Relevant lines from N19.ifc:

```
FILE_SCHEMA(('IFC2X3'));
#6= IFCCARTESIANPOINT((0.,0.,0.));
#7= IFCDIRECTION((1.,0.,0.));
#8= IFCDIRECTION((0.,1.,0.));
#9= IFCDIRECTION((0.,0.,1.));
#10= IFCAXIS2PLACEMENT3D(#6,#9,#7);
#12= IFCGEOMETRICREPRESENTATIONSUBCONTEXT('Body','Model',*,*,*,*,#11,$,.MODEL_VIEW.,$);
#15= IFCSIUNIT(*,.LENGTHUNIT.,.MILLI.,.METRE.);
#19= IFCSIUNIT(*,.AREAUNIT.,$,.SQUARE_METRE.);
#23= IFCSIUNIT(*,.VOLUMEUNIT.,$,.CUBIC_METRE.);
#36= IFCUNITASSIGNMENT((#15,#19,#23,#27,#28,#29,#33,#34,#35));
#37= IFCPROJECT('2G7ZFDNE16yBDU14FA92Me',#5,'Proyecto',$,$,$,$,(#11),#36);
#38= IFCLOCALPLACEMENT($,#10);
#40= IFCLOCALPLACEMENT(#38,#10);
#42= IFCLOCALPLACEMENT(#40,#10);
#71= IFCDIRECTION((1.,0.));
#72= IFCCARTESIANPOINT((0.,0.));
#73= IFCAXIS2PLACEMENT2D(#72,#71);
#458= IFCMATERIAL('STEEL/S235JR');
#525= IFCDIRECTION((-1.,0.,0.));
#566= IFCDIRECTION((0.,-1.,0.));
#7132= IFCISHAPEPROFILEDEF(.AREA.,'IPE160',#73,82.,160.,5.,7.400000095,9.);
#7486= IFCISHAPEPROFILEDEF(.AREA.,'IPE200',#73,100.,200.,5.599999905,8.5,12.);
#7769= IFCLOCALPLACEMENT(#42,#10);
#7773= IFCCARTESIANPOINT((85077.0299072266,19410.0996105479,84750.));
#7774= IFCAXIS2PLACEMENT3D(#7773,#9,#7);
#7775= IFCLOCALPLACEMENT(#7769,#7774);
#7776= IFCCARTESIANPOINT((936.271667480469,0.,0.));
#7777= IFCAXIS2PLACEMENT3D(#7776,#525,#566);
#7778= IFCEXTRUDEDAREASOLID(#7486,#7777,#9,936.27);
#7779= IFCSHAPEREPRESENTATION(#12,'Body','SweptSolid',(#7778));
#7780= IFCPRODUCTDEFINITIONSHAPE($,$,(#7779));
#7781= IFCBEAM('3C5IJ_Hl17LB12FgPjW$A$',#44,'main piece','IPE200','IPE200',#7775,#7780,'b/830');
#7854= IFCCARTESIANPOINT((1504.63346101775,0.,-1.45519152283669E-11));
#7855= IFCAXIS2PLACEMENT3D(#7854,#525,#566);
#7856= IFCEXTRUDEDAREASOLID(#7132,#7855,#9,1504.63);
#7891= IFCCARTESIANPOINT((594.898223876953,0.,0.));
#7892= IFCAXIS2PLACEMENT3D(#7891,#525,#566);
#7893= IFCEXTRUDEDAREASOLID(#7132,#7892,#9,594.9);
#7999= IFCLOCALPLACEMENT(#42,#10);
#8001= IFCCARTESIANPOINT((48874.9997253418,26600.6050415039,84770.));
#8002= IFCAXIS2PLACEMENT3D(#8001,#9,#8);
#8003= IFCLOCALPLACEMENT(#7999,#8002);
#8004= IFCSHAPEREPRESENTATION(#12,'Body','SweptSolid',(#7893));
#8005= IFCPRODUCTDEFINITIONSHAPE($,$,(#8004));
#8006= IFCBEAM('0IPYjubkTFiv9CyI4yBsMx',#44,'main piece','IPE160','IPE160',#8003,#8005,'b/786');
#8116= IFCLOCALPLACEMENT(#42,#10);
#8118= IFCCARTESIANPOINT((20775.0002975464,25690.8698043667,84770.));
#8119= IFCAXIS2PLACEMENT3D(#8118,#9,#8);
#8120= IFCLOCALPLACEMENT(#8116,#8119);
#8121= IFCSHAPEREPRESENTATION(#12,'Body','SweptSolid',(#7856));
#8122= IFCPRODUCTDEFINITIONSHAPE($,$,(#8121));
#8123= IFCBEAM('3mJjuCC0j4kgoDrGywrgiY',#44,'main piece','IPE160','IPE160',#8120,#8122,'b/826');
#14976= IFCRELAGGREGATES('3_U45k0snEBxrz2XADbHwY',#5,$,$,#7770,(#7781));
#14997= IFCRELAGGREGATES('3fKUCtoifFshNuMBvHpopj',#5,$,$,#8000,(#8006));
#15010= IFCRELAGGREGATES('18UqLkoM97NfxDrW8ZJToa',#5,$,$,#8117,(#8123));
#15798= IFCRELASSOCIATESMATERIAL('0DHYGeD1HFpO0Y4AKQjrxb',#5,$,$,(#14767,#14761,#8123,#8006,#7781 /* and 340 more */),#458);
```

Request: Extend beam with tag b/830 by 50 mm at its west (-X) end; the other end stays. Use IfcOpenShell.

```python
import ifcopenshell
import ifcopenshell.util.representation

model = ifcopenshell.open("N19.ifc")

member = model.by_id(7781)
change = 50.0

# The extrusion runs towards the end named, so only its depth changes.
body = ifcopenshell.util.representation.get_representation(member, "Model", "Body")
solid = body.Items[0]
old_length = solid.Depth
solid.Depth += change

print(f"length {old_length:g} -> {solid.Depth:g}")

model.write("N19_rev.ifc")
```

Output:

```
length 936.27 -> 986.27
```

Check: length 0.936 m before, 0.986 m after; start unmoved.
